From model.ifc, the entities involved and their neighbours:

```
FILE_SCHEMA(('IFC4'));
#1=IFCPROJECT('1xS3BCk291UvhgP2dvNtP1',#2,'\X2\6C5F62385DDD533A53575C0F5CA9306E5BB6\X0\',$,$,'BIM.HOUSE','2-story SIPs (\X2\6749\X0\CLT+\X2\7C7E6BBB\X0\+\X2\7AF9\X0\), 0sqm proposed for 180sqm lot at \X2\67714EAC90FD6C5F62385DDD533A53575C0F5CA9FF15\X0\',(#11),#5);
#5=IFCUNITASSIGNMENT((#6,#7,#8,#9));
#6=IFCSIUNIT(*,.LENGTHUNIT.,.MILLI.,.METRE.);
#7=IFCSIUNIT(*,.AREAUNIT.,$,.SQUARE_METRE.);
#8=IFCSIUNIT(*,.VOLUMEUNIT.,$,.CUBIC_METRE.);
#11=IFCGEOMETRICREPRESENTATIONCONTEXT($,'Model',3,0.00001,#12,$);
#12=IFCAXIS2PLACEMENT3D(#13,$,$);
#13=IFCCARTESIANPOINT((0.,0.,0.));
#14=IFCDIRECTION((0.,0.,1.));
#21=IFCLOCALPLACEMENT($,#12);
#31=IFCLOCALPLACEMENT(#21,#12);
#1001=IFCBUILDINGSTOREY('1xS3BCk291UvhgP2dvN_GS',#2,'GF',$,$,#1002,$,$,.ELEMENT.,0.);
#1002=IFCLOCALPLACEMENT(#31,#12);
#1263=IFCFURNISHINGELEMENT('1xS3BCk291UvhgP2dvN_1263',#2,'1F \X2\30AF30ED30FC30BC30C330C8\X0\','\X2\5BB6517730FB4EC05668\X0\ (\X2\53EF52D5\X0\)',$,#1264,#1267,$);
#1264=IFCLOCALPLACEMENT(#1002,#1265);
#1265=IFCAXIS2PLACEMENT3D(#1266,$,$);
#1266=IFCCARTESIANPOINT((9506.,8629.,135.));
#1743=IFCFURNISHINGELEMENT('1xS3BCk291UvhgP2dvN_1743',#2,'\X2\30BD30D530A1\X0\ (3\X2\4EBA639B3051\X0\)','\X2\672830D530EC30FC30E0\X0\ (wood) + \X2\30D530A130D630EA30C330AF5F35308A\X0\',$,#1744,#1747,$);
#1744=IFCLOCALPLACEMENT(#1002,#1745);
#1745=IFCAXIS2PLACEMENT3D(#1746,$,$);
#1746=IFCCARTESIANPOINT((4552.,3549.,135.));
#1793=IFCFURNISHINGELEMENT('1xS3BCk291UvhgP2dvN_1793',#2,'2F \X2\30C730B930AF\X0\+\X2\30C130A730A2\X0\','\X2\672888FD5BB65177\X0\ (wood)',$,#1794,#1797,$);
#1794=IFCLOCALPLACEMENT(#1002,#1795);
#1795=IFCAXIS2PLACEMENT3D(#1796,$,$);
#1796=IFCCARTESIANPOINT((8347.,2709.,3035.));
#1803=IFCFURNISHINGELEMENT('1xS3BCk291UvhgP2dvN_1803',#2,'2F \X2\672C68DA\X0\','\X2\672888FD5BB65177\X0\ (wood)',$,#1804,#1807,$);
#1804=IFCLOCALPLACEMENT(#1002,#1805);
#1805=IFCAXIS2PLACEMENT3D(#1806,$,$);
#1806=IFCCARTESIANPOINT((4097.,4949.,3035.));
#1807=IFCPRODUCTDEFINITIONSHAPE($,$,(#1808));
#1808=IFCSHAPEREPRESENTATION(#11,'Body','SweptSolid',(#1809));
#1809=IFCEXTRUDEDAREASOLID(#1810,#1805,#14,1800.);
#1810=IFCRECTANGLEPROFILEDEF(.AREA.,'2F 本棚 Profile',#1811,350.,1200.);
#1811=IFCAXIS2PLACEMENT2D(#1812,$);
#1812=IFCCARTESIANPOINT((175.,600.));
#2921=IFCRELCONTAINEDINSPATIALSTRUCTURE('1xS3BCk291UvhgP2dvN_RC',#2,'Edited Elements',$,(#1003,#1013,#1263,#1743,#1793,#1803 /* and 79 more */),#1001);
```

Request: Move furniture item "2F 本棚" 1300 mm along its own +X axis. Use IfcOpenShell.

```python
import ifcopenshell
import ifcopenshell.api.geometry
import ifcopenshell.util.placement
import ifcopenshell.util.unit

model = ifcopenshell.open("model.ifc")
unit_scale = ifcopenshell.util.unit.calculate_unit_scale(model)

item = model.by_guid("1xS3BCk291UvhgP2dvN_1803")
matrix = ifcopenshell.util.placement.get_local_placement(item.ObjectPlacement)
matrix[:3, 3] += matrix[:3, 0] * 1.3 / unit_scale
ifcopenshell.api.geometry.edit_object_placement(model, product=item, matrix=matrix, is_si=False)

print(ifcopenshell.util.placement.get_local_placement(item.ObjectPlacement).round(3) + 0.0)

model.write("model_rev.ifc")
```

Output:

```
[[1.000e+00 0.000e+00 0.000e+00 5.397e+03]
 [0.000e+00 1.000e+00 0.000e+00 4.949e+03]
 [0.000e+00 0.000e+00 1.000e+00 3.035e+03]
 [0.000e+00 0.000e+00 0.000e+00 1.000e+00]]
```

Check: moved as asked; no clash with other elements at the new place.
